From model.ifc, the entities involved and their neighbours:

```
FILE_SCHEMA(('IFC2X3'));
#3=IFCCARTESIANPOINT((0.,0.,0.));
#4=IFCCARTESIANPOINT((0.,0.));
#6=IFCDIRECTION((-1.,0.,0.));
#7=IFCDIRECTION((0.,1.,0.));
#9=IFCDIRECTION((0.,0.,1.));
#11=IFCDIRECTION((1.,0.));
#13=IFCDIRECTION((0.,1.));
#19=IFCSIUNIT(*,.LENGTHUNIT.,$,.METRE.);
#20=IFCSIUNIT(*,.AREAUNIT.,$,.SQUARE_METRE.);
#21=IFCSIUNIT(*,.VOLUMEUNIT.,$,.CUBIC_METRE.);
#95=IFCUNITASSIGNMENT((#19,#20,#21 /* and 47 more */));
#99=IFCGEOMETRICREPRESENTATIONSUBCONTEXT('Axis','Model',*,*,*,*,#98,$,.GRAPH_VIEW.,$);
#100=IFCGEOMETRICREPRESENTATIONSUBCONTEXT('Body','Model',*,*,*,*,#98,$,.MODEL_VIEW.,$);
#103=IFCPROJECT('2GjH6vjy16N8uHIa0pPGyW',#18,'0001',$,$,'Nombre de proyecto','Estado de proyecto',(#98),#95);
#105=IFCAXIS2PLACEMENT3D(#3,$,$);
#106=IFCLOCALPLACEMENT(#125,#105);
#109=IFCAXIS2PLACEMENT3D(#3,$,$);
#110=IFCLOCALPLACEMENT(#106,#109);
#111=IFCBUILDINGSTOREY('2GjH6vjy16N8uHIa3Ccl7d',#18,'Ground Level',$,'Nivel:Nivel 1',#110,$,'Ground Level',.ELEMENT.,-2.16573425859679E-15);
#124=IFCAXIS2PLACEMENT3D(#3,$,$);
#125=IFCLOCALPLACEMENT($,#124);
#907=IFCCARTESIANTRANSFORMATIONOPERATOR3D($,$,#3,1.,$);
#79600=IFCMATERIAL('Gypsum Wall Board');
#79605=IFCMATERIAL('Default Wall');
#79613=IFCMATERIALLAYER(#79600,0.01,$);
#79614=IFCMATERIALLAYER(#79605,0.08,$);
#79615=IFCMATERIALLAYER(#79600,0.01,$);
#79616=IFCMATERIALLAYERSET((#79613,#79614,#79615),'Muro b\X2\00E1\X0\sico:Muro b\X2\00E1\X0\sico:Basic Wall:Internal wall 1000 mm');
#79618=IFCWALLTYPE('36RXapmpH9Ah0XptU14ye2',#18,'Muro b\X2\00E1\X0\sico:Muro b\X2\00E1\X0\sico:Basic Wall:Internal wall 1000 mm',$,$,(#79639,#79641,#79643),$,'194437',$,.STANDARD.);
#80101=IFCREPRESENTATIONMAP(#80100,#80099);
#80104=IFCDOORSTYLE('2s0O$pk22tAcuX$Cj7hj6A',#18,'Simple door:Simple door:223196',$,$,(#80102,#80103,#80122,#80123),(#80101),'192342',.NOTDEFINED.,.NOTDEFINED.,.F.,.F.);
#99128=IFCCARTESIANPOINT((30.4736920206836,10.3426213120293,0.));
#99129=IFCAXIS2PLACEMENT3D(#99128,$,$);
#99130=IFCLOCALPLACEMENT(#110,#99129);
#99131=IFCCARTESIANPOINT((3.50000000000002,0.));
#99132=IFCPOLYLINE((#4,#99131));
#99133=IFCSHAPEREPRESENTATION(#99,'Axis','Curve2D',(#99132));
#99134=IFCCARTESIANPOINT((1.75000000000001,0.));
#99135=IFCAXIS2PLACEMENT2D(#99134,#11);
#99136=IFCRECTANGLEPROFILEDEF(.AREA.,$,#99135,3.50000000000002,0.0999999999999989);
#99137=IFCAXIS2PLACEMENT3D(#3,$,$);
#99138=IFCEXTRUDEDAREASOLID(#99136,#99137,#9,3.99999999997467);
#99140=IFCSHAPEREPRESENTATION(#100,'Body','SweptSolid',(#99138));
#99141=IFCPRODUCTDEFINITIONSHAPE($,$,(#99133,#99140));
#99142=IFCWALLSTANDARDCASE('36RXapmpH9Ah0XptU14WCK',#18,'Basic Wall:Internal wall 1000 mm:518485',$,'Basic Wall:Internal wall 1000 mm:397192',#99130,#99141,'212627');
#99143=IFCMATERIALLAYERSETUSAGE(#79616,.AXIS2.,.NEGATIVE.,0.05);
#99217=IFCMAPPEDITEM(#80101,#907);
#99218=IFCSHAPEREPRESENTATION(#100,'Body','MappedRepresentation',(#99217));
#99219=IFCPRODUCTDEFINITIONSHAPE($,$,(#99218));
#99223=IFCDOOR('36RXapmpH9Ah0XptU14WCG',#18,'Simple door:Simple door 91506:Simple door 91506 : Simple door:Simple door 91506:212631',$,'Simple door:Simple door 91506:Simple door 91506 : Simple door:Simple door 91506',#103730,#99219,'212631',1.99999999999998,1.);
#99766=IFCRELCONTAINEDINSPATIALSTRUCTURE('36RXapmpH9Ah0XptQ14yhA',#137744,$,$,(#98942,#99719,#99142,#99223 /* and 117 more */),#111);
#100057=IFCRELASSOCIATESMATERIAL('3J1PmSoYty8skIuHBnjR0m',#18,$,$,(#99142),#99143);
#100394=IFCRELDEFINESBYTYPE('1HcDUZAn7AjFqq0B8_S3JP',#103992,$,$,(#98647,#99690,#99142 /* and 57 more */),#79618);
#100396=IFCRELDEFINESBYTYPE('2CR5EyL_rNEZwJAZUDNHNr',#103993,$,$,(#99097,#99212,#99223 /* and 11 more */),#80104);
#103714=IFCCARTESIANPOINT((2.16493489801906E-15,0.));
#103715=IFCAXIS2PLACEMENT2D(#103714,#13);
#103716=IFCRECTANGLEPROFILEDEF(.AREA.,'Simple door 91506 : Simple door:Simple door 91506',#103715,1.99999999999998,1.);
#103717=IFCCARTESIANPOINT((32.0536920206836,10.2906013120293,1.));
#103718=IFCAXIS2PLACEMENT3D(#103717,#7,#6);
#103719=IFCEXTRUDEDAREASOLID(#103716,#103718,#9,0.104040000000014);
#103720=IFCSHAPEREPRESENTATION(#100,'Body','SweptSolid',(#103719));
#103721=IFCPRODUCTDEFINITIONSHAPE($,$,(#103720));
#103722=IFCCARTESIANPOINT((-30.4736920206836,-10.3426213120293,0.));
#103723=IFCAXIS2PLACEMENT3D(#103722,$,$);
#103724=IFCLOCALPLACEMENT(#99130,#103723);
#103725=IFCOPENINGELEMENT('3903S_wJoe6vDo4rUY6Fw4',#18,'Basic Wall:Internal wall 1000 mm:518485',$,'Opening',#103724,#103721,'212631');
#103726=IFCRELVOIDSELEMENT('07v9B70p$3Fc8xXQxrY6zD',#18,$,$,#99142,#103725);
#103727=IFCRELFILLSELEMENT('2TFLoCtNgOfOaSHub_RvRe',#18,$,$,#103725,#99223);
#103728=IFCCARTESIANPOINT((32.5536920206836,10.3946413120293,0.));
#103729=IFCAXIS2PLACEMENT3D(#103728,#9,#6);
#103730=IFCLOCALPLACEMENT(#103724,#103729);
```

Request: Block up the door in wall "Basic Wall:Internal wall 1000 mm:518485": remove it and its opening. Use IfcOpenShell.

```python
import ifcopenshell
import ifcopenshell.api.feature
import ifcopenshell.api.root
import ifcopenshell.geom
import ifcopenshell.util.shape

model = ifcopenshell.open("model.ifc")
settings = ifcopenshell.geom.settings()


def volume(element):
    """Net volume in cubic metres, openings subtracted."""
    shape = ifcopenshell.geom.create_shape(settings, element)
    return ifcopenshell.util.shape.get_volume(shape.geometry)


door = model.by_id(99223)
opening = door.FillsVoids[0].RelatingOpeningElement
wall = opening.VoidsElements[0].RelatingBuildingElement
before = volume(wall)

ifcopenshell.api.root.remove_product(model, product=door)
ifcopenshell.api.feature.remove_feature(model, feature=opening)

after = volume(wall)

print(f"wall volume {before:.3f} -> {after:.3f} m3")

model.write("model_v2.ifc")
```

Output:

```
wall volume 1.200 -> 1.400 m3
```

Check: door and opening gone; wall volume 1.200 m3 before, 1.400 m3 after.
